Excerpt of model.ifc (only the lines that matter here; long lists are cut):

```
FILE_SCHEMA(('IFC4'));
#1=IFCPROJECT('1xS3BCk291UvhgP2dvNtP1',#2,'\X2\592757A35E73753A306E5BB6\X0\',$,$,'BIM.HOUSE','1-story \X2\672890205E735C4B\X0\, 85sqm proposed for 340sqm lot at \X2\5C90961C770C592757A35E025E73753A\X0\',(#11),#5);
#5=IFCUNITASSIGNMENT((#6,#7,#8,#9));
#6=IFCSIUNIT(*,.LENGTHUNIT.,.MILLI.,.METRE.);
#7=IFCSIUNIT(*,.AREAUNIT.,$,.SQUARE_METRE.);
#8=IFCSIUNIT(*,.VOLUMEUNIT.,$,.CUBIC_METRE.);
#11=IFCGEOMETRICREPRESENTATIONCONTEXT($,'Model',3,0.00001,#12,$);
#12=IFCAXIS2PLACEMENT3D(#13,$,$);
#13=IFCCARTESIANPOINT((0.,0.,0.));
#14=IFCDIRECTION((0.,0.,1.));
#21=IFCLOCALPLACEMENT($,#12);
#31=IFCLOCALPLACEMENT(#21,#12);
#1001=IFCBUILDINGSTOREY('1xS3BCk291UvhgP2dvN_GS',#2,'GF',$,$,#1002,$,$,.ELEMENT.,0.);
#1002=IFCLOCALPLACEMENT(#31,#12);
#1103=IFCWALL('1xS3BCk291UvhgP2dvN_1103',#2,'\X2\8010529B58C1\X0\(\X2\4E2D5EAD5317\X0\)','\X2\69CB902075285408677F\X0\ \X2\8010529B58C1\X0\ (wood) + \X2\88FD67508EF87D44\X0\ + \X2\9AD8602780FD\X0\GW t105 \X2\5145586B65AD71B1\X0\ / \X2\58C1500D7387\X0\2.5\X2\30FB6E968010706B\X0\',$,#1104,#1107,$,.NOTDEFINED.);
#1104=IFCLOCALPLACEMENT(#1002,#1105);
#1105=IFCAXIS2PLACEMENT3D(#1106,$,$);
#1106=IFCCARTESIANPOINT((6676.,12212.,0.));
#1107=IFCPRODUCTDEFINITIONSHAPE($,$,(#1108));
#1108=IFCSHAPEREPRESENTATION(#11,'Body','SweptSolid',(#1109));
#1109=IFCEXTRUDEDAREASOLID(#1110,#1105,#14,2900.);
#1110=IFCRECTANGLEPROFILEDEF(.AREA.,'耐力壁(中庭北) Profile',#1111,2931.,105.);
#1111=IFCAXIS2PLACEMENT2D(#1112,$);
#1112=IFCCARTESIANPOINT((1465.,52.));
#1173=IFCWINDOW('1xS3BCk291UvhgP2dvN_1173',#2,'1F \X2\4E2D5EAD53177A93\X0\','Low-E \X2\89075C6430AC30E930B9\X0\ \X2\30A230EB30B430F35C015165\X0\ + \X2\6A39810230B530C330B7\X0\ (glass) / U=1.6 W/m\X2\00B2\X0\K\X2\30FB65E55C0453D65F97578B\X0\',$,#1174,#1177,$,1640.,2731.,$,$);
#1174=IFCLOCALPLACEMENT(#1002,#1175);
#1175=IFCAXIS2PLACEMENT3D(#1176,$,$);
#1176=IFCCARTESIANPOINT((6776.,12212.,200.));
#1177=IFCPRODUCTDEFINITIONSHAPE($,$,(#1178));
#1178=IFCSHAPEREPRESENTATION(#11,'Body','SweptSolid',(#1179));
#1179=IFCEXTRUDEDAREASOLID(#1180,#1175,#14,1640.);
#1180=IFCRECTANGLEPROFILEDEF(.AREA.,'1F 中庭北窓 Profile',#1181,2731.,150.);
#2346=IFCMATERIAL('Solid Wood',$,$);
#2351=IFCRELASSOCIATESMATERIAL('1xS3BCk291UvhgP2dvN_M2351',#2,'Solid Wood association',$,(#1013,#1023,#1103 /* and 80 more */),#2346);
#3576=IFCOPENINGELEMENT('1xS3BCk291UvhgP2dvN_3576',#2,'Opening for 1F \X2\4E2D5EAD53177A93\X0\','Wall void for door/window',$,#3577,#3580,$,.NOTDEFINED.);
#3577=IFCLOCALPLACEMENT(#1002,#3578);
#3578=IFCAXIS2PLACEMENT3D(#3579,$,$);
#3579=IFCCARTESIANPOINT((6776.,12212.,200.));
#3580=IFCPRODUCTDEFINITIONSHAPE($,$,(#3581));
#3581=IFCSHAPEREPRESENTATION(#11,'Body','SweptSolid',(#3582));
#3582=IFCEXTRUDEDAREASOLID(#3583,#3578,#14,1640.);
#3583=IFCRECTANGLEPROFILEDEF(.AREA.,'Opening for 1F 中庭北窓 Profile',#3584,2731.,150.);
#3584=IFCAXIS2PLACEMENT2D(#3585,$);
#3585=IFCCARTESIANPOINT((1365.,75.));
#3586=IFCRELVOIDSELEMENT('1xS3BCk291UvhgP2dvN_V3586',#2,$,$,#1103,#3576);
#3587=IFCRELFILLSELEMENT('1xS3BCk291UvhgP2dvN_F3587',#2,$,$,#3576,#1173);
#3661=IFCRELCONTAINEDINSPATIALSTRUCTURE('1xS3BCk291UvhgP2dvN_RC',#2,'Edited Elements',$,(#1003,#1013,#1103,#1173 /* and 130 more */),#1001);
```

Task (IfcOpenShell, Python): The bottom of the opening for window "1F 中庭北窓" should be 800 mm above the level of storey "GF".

```python
import numpy as np
import ifcopenshell
import ifcopenshell.api.geometry
import ifcopenshell.geom
import ifcopenshell.util.element
import ifcopenshell.util.placement
import ifcopenshell.util.shape
import ifcopenshell.util.unit

model = ifcopenshell.open("model.ifc")
unit_scale = ifcopenshell.util.unit.calculate_unit_scale(model)

window = model.by_guid("1xS3BCk291UvhgP2dvN_1173")
opening = window.FillsVoids[0].RelatingOpeningElement
storey = ifcopenshell.util.element.get_container(window, ifc_class="IfcBuildingStorey")
level = ifcopenshell.util.placement.get_local_placement(storey.ObjectPlacement)[2, 3]

# The opening's origin need not be at the sill, so measure its lowest point.
shape = ifcopenshell.geom.create_shape(ifcopenshell.geom.settings(), opening)
bottom = ifcopenshell.util.shape.get_shape_bottom_elevation(shape, shape.geometry) / unit_scale
dz = level + 0.8 / unit_scale - bottom

shift = np.array([0.0, 0.0, dz])
# The window is not placed relative to its opening, so move both.
for product in (opening, window):
    matrix = ifcopenshell.util.placement.get_local_placement(product.ObjectPlacement)
    matrix[:3, 3] += shift
    ifcopenshell.api.geometry.edit_object_placement(model, product=product, matrix=matrix, is_si=False)

print(f"moved by {dz * unit_scale:+.3f} m")

model.write("model_updated.ifc")
```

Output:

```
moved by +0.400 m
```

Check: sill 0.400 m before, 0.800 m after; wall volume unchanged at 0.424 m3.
